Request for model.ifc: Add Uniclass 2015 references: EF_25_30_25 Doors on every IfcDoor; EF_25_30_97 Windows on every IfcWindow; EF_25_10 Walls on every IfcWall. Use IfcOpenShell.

First a look at what the model holds.

```python
import ifcopenshell

model = ifcopenshell.open("model.ifc")
print(model.schema)
print("classifications:", [c.Name for c in model.by_type("IfcClassification")])
for ifc_class in ("IfcDoor", "IfcRoof", "IfcStair", "IfcWall", "IfcWindow"):
    print(ifc_class, len(model.by_type(ifc_class)))
```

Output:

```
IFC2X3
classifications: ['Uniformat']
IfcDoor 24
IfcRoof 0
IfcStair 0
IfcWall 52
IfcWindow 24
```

```python
import ifcopenshell
import ifcopenshell.api.classification

model = ifcopenshell.open("model.ifc")

# IFC2X3 requires Source and Edition and has no link from the project to the system.
system = model.create_entity("IfcClassification", Source="NBS", Edition="2015", Name="Uniclass 2015")

codes = {
    "IfcDoor": ("EF_25_30_25", "Doors"),
    "IfcWindow": ("EF_25_30_97", "Windows"),
    "IfcWall": ("EF_25_10", "Walls"),
}
for ifc_class, (code, name) in codes.items():
    products = model.by_type(ifc_class)
    ifcopenshell.api.classification.add_reference(
        model, products=products, classification=system, identification=code, name=name
    )
    print(code, len(products))

model.write("model_rev.ifc")
```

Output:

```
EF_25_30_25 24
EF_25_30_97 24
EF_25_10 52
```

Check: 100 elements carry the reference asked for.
